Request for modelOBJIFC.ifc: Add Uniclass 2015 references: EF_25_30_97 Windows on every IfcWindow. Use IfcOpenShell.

First a look at what the model holds.

```python
import ifcopenshell

model = ifcopenshell.open("modelOBJIFC.ifc")
print(model.schema)
print("classifications:", [c.Name for c in model.by_type("IfcClassification")])
for ifc_class in ("IfcDoor", "IfcRoof", "IfcStair", "IfcWall", "IfcWindow"):
    print(ifc_class, len(model.by_type(ifc_class)))
```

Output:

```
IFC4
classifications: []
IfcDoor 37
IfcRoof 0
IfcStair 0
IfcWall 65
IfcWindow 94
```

```python
import ifcopenshell
import ifcopenshell.api.classification

model = ifcopenshell.open("modelOBJIFC.ifc")

system = ifcopenshell.api.classification.add_classification(model, classification="Uniclass 2015")

codes = {
    "IfcWindow": ("EF_25_30_97", "Windows"),
}
for ifc_class, (code, name) in codes.items():
    products = model.by_type(ifc_class)
    ifcopenshell.api.classification.add_reference(
        model, products=products, classification=system, identification=code, name=name
    )
    print(code, len(products))

model.write("modelOBJIFC_updated.ifc")
```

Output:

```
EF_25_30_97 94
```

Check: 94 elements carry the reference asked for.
